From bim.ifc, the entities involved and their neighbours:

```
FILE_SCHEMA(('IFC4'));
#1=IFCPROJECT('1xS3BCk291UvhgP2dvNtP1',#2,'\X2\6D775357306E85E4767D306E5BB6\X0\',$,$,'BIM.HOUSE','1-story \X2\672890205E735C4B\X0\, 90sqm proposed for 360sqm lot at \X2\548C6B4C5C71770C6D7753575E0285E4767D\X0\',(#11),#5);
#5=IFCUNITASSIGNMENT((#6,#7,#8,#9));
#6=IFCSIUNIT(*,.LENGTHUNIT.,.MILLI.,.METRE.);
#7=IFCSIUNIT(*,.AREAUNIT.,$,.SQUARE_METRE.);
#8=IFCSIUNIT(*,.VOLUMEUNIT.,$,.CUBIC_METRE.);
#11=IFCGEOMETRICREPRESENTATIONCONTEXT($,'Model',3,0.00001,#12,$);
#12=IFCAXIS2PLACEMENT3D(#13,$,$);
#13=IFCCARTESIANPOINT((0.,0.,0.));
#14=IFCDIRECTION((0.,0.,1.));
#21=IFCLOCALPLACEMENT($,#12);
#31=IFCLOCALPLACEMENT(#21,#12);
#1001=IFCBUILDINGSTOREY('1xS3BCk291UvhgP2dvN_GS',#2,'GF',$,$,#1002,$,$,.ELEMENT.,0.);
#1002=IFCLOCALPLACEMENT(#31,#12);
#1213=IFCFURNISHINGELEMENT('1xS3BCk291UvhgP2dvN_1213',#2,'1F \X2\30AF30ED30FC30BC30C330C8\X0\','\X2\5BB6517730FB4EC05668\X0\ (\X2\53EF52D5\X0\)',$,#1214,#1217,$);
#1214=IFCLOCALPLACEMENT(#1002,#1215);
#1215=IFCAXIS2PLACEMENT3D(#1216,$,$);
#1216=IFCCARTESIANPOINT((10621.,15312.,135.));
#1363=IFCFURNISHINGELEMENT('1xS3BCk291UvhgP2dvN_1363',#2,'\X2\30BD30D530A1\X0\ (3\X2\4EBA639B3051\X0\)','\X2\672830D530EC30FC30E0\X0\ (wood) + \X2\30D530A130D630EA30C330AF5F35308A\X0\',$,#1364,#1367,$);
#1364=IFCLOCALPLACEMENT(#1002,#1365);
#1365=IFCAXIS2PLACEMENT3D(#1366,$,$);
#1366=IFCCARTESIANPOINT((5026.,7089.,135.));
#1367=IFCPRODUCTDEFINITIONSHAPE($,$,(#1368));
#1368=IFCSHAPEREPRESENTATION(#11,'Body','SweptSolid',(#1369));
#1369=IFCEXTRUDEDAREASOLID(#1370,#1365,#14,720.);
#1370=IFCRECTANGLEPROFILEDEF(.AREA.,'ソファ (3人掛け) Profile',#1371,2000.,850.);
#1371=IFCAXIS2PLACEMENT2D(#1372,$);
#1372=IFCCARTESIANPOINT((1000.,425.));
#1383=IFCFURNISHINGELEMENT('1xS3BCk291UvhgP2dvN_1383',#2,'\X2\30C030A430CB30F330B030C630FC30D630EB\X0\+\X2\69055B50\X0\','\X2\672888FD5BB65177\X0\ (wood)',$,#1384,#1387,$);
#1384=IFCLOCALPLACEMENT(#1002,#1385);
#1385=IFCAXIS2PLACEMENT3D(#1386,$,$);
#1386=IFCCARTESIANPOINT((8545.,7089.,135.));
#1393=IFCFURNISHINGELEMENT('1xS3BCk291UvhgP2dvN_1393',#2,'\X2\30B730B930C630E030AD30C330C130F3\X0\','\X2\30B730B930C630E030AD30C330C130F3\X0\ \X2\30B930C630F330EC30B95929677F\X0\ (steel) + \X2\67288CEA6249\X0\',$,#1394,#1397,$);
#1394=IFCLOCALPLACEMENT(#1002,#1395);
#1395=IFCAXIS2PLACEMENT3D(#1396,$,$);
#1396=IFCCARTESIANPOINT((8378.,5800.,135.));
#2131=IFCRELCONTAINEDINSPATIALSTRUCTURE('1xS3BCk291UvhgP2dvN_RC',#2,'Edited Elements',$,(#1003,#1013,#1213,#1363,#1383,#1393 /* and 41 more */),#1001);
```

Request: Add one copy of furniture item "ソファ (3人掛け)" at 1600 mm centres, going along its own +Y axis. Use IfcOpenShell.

```python
import ifcopenshell
import ifcopenshell.api.geometry
import ifcopenshell.api.root
import ifcopenshell.util.element
import ifcopenshell.util.placement
import ifcopenshell.util.unit

model = ifcopenshell.open("bim.ifc")
unit_scale = ifcopenshell.util.unit.calculate_unit_scale(model)


def reuse_history(source, copy):
    """copy_class also copies each property set's owner history, people and application; keep the originals."""
    for rel in copy.IsDefinedBy:
        if rel.is_a("IfcRelDefinesByProperties") and (history := rel.RelatingPropertyDefinition.OwnerHistory):
            rel.RelatingPropertyDefinition.OwnerHistory = source.OwnerHistory
            ifcopenshell.util.element.remove_deep2(model, history)


source = model.by_guid("1xS3BCk291UvhgP2dvN_1363")
base = ifcopenshell.util.placement.get_local_placement(source.ObjectPlacement)
step = base[:3, 1] * 1.6 / unit_scale

for i in range(1, 2):
    copy = ifcopenshell.api.root.copy_class(model, product=source)
    copy.Representation = ifcopenshell.util.element.copy_deep(
        model, source.Representation, exclude=["IfcGeometricRepresentationContext", "IfcRepresentationMap"]
    )
    reuse_history(source, copy)
    matrix = base.copy()
    matrix[:3, 3] += i * step
    print("added at", matrix[:3, 3].round(3) + 0.0)
    ifcopenshell.api.geometry.edit_object_placement(model, product=copy, matrix=matrix, is_si=False)

model.write("bim_rev.ifc")
```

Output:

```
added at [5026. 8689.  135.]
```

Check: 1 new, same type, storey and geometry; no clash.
